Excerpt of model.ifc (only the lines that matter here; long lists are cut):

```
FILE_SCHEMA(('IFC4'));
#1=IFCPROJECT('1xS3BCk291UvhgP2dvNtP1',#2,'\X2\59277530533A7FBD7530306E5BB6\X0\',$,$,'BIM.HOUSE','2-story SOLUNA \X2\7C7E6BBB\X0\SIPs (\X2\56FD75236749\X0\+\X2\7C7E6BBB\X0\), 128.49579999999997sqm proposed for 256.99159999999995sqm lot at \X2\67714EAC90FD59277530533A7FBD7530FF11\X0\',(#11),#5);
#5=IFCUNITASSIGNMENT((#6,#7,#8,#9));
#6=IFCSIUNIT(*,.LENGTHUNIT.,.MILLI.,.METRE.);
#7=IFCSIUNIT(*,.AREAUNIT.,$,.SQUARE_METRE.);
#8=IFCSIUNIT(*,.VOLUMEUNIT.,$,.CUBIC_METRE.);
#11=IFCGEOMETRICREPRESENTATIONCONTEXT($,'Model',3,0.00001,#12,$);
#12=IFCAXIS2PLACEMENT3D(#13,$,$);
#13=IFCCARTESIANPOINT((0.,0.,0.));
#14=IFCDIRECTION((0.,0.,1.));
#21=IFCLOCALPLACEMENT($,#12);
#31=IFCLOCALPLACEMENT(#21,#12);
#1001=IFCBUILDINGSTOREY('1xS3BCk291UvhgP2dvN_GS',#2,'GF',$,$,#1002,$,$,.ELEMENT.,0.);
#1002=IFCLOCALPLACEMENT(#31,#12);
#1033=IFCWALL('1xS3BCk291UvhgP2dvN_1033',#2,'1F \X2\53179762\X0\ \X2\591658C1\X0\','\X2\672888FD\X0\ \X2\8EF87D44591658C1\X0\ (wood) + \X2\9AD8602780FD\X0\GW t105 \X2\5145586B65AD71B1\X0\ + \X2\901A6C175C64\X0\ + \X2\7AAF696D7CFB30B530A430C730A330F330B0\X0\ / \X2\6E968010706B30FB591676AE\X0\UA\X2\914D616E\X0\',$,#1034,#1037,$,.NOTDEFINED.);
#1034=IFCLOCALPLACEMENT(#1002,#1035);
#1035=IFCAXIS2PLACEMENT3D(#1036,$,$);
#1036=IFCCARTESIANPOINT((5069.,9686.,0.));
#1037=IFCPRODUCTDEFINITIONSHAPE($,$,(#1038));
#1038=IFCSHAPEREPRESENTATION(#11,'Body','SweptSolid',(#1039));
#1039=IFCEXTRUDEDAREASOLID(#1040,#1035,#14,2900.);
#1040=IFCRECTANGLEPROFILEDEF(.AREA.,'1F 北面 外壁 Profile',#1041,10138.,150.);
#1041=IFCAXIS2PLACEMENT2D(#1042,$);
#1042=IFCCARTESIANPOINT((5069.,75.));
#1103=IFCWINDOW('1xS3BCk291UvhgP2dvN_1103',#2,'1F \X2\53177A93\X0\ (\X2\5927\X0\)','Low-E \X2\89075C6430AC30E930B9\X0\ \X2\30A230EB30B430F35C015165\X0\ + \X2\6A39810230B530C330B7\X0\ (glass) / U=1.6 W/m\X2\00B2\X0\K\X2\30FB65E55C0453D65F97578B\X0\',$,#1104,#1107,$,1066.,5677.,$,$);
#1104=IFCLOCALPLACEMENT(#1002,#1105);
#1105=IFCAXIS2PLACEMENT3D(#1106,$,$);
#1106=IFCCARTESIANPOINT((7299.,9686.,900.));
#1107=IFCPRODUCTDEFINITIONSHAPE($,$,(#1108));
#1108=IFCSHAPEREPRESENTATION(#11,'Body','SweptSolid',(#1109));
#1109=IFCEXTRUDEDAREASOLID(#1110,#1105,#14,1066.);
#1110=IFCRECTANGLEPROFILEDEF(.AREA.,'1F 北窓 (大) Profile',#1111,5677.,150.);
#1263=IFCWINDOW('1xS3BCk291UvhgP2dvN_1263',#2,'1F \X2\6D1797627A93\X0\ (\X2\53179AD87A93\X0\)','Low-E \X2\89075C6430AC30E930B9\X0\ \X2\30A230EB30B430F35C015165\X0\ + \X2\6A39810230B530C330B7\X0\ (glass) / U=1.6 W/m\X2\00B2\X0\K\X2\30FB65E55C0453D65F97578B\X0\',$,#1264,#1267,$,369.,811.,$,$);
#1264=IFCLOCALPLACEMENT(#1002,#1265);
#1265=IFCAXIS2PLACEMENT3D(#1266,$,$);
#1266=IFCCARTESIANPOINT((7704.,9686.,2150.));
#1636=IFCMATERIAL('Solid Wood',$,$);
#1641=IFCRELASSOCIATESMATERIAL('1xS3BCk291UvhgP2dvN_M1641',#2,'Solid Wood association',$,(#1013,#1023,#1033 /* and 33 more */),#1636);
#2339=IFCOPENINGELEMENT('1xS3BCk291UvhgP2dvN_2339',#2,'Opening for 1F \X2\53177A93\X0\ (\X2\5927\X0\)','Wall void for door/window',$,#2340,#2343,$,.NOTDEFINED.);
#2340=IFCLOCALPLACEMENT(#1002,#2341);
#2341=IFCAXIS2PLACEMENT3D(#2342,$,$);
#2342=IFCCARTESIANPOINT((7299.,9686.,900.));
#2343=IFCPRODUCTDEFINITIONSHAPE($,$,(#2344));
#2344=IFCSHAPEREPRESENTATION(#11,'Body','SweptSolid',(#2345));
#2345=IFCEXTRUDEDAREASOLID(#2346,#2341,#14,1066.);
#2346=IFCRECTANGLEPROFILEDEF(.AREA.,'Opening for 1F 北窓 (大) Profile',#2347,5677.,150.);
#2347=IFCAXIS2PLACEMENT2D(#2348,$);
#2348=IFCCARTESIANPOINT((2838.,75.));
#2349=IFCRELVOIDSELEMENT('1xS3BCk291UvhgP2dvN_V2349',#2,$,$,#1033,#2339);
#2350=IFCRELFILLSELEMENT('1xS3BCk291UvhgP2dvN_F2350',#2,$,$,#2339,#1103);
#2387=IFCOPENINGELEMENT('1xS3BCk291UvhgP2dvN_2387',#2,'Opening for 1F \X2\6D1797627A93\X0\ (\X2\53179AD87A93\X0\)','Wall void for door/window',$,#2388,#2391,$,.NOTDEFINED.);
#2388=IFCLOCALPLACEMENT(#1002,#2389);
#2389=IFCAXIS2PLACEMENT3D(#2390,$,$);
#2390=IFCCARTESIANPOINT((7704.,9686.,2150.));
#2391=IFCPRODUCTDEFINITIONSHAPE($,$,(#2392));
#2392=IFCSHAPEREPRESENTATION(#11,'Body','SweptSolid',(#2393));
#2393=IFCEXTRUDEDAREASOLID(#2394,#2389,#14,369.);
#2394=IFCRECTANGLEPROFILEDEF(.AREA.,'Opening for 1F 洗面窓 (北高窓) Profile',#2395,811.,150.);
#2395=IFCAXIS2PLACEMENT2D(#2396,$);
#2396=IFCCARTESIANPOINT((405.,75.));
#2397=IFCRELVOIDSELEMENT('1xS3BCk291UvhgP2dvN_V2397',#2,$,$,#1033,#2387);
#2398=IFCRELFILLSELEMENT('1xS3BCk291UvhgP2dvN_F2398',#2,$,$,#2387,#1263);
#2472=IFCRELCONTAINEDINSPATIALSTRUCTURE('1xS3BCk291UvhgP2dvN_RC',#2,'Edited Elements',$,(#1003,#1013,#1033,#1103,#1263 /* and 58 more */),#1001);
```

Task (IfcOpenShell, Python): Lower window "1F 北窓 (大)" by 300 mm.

```python
import numpy as np
import ifcopenshell
import ifcopenshell.api.geometry
import ifcopenshell.util.placement
import ifcopenshell.util.unit

model = ifcopenshell.open("model.ifc")
unit_scale = ifcopenshell.util.unit.calculate_unit_scale(model)

window = model.by_guid("1xS3BCk291UvhgP2dvN_1103")
opening = window.FillsVoids[0].RelatingOpeningElement
dz = -0.3 / unit_scale

shift = np.array([0.0, 0.0, dz])
# The window is not placed relative to its opening, so move both.
for product in (opening, window):
    matrix = ifcopenshell.util.placement.get_local_placement(product.ObjectPlacement)
    matrix[:3, 3] += shift
    ifcopenshell.api.geometry.edit_object_placement(model, product=product, matrix=matrix, is_si=False)

print(f"moved by {dz * unit_scale:+.3f} m")

model.write("model_rev.ifc")
```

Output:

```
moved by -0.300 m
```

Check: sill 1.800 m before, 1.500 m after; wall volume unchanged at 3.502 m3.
